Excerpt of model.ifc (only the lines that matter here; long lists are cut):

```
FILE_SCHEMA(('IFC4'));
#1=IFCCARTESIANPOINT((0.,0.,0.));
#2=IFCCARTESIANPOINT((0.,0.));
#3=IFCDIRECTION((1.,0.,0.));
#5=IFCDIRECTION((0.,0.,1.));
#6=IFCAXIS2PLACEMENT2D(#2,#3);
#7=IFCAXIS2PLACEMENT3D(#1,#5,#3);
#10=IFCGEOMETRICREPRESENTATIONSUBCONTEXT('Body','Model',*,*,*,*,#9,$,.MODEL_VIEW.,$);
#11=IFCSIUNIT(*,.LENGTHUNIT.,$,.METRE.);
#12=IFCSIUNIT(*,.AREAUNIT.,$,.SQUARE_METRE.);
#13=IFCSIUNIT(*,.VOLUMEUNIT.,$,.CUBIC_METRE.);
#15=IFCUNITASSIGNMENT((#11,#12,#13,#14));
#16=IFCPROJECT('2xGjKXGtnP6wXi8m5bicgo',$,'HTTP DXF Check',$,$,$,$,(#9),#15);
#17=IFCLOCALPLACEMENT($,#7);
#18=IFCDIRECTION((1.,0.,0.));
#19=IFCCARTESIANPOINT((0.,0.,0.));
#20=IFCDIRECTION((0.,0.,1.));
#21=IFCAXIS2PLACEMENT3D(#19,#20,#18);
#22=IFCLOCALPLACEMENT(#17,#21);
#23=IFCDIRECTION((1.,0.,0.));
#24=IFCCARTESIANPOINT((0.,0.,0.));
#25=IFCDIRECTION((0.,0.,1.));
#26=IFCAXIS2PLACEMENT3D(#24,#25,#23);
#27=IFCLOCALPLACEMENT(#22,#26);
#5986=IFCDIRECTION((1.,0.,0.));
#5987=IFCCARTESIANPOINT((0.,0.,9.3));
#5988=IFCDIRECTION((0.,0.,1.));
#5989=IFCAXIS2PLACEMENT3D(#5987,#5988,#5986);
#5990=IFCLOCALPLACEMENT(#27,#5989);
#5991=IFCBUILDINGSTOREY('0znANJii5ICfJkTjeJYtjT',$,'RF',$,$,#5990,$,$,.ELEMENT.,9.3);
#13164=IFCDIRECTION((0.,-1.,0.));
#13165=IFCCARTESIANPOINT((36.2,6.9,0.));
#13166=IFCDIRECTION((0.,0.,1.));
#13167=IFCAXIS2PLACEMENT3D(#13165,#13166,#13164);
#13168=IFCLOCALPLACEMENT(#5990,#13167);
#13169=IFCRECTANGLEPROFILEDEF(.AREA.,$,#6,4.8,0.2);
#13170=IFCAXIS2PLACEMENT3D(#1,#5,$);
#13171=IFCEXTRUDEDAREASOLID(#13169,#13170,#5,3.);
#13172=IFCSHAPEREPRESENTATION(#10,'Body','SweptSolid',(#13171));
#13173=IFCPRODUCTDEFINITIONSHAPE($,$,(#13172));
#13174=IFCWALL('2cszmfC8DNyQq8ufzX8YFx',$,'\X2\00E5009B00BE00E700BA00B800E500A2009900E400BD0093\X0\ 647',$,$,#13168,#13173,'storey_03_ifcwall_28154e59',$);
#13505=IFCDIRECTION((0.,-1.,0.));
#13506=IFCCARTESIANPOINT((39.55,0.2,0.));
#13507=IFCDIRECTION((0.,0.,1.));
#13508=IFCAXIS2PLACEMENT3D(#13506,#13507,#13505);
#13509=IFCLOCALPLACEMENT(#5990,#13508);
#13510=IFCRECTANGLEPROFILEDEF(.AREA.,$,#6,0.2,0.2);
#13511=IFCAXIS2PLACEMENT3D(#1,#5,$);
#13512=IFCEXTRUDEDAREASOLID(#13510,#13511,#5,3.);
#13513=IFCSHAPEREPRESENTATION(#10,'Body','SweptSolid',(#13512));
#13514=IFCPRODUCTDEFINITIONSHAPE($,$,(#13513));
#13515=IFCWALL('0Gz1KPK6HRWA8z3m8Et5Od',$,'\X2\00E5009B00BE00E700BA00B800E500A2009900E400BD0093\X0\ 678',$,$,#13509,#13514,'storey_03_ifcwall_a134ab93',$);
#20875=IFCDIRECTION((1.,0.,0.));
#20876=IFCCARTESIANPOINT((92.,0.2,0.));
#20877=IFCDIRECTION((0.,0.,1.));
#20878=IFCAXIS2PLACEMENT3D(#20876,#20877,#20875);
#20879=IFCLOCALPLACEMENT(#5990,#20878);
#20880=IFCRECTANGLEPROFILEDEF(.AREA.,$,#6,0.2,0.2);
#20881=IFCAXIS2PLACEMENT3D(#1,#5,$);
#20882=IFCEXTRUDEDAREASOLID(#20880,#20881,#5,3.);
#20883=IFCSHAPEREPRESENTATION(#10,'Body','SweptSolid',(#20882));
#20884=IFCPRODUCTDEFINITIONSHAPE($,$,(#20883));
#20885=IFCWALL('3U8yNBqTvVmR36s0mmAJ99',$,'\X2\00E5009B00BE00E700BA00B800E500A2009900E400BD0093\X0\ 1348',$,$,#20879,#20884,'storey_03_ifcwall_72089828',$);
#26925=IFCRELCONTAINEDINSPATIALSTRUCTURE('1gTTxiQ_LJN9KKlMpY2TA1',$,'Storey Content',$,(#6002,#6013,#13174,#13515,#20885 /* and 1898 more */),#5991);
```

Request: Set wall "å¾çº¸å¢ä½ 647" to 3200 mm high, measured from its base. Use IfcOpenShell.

```python
import ifcopenshell
import ifcopenshell.geom
import ifcopenshell.util.representation
import ifcopenshell.util.shape
import ifcopenshell.util.unit

model = ifcopenshell.open("model.ifc")
unit_scale = ifcopenshell.util.unit.calculate_unit_scale(model)
settings = ifcopenshell.geom.settings()


def volume(element):
    """Net volume in cubic metres, openings subtracted."""
    shape = ifcopenshell.geom.create_shape(settings, element)
    return ifcopenshell.util.shape.get_volume(shape.geometry)


wall = model.by_guid("2cszmfC8DNyQq8ufzX8YFx")
before = volume(wall)

body = ifcopenshell.util.representation.get_representation(wall, "Model", "Body")
solid = body.Items[0]
old_height = solid.Depth
solid.Depth = 3.2 / unit_scale
after = volume(wall)

print(f"height {old_height:g} -> {solid.Depth:g}, volume {before:.3f} -> {after:.3f} m3")

model.write("model_edited.ifc")
```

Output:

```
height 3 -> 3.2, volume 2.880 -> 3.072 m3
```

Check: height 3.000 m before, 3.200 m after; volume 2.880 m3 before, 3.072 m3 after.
